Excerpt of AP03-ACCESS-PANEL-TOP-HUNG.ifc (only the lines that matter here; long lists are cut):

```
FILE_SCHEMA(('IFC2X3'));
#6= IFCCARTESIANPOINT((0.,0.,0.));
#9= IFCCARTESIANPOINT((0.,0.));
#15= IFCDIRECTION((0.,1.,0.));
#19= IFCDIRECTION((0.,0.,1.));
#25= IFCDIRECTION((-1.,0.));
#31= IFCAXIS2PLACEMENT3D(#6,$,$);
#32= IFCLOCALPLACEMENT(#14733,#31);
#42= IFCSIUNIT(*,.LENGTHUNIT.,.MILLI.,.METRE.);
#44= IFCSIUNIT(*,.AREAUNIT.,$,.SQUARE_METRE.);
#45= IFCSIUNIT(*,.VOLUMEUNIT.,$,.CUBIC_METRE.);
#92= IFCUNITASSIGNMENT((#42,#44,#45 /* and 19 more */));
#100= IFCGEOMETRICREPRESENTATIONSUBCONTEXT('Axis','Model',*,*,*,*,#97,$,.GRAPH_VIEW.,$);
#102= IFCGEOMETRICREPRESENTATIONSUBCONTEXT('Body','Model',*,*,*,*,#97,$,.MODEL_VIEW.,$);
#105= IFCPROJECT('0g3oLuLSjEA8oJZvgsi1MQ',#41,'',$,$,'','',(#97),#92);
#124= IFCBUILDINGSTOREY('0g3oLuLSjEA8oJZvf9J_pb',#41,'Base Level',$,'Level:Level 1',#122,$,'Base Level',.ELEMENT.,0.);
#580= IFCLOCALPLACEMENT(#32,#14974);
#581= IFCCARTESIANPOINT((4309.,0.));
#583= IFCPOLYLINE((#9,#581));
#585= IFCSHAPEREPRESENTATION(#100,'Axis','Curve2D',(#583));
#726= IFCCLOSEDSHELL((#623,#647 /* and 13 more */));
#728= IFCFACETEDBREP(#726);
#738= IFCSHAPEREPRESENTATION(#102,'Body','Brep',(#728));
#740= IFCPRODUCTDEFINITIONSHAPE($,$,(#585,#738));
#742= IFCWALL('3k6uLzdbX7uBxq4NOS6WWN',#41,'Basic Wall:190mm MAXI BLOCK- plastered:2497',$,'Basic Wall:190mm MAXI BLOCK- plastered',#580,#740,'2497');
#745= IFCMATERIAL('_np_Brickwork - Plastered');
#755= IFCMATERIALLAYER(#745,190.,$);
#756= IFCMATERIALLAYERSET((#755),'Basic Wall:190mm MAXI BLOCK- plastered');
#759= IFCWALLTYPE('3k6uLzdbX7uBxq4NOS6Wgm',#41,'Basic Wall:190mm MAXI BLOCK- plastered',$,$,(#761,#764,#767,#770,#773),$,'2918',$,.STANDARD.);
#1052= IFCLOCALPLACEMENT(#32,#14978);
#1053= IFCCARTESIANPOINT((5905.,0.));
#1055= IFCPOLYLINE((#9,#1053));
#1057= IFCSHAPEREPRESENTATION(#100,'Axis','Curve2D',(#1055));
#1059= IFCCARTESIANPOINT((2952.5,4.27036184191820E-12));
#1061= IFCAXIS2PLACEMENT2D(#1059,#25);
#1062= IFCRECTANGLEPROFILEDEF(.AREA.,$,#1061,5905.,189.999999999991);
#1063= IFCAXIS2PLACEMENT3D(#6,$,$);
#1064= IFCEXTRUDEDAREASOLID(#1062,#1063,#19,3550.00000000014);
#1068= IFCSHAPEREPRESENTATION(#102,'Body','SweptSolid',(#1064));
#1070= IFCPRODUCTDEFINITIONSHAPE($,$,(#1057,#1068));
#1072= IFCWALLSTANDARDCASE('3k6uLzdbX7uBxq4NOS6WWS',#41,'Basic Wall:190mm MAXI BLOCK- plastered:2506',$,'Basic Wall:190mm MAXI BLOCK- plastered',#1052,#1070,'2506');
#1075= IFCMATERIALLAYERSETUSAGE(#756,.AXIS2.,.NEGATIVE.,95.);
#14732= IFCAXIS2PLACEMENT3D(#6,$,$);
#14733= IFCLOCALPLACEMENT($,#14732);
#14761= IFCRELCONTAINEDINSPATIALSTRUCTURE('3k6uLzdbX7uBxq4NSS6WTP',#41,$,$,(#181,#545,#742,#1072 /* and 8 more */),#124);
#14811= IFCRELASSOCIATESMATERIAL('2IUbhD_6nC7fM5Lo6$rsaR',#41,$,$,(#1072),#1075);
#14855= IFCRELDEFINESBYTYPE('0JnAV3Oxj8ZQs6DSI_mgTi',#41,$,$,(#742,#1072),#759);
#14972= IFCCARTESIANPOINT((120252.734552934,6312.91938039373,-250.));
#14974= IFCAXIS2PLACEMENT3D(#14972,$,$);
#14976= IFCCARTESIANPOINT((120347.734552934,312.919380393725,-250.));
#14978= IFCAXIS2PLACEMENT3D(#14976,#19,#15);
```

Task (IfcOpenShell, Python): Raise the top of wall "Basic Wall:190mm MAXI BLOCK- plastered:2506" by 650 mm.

```python
import ifcopenshell
import ifcopenshell.geom
import ifcopenshell.util.representation
import ifcopenshell.util.shape
import ifcopenshell.util.unit

model = ifcopenshell.open("AP03-ACCESS-PANEL-TOP-HUNG.ifc")
unit_scale = ifcopenshell.util.unit.calculate_unit_scale(model)
settings = ifcopenshell.geom.settings()


def volume(element):
    """Net volume in cubic metres, openings subtracted."""
    shape = ifcopenshell.geom.create_shape(settings, element)
    return ifcopenshell.util.shape.get_volume(shape.geometry)


wall = model.by_guid("3k6uLzdbX7uBxq4NOS6WWS")
before = volume(wall)

body = ifcopenshell.util.representation.get_representation(wall, "Model", "Body")
solid = body.Items[0]
old_height = solid.Depth
solid.Depth += 0.65 / unit_scale
after = volume(wall)

print(f"height {old_height:g} -> {solid.Depth:g}, volume {before:.3f} -> {after:.3f} m3")

model.write("AP03-ACCESS-PANEL-TOP-HUNG_rev.ifc")
```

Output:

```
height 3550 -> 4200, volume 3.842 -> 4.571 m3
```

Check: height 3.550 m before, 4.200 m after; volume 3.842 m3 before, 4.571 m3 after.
